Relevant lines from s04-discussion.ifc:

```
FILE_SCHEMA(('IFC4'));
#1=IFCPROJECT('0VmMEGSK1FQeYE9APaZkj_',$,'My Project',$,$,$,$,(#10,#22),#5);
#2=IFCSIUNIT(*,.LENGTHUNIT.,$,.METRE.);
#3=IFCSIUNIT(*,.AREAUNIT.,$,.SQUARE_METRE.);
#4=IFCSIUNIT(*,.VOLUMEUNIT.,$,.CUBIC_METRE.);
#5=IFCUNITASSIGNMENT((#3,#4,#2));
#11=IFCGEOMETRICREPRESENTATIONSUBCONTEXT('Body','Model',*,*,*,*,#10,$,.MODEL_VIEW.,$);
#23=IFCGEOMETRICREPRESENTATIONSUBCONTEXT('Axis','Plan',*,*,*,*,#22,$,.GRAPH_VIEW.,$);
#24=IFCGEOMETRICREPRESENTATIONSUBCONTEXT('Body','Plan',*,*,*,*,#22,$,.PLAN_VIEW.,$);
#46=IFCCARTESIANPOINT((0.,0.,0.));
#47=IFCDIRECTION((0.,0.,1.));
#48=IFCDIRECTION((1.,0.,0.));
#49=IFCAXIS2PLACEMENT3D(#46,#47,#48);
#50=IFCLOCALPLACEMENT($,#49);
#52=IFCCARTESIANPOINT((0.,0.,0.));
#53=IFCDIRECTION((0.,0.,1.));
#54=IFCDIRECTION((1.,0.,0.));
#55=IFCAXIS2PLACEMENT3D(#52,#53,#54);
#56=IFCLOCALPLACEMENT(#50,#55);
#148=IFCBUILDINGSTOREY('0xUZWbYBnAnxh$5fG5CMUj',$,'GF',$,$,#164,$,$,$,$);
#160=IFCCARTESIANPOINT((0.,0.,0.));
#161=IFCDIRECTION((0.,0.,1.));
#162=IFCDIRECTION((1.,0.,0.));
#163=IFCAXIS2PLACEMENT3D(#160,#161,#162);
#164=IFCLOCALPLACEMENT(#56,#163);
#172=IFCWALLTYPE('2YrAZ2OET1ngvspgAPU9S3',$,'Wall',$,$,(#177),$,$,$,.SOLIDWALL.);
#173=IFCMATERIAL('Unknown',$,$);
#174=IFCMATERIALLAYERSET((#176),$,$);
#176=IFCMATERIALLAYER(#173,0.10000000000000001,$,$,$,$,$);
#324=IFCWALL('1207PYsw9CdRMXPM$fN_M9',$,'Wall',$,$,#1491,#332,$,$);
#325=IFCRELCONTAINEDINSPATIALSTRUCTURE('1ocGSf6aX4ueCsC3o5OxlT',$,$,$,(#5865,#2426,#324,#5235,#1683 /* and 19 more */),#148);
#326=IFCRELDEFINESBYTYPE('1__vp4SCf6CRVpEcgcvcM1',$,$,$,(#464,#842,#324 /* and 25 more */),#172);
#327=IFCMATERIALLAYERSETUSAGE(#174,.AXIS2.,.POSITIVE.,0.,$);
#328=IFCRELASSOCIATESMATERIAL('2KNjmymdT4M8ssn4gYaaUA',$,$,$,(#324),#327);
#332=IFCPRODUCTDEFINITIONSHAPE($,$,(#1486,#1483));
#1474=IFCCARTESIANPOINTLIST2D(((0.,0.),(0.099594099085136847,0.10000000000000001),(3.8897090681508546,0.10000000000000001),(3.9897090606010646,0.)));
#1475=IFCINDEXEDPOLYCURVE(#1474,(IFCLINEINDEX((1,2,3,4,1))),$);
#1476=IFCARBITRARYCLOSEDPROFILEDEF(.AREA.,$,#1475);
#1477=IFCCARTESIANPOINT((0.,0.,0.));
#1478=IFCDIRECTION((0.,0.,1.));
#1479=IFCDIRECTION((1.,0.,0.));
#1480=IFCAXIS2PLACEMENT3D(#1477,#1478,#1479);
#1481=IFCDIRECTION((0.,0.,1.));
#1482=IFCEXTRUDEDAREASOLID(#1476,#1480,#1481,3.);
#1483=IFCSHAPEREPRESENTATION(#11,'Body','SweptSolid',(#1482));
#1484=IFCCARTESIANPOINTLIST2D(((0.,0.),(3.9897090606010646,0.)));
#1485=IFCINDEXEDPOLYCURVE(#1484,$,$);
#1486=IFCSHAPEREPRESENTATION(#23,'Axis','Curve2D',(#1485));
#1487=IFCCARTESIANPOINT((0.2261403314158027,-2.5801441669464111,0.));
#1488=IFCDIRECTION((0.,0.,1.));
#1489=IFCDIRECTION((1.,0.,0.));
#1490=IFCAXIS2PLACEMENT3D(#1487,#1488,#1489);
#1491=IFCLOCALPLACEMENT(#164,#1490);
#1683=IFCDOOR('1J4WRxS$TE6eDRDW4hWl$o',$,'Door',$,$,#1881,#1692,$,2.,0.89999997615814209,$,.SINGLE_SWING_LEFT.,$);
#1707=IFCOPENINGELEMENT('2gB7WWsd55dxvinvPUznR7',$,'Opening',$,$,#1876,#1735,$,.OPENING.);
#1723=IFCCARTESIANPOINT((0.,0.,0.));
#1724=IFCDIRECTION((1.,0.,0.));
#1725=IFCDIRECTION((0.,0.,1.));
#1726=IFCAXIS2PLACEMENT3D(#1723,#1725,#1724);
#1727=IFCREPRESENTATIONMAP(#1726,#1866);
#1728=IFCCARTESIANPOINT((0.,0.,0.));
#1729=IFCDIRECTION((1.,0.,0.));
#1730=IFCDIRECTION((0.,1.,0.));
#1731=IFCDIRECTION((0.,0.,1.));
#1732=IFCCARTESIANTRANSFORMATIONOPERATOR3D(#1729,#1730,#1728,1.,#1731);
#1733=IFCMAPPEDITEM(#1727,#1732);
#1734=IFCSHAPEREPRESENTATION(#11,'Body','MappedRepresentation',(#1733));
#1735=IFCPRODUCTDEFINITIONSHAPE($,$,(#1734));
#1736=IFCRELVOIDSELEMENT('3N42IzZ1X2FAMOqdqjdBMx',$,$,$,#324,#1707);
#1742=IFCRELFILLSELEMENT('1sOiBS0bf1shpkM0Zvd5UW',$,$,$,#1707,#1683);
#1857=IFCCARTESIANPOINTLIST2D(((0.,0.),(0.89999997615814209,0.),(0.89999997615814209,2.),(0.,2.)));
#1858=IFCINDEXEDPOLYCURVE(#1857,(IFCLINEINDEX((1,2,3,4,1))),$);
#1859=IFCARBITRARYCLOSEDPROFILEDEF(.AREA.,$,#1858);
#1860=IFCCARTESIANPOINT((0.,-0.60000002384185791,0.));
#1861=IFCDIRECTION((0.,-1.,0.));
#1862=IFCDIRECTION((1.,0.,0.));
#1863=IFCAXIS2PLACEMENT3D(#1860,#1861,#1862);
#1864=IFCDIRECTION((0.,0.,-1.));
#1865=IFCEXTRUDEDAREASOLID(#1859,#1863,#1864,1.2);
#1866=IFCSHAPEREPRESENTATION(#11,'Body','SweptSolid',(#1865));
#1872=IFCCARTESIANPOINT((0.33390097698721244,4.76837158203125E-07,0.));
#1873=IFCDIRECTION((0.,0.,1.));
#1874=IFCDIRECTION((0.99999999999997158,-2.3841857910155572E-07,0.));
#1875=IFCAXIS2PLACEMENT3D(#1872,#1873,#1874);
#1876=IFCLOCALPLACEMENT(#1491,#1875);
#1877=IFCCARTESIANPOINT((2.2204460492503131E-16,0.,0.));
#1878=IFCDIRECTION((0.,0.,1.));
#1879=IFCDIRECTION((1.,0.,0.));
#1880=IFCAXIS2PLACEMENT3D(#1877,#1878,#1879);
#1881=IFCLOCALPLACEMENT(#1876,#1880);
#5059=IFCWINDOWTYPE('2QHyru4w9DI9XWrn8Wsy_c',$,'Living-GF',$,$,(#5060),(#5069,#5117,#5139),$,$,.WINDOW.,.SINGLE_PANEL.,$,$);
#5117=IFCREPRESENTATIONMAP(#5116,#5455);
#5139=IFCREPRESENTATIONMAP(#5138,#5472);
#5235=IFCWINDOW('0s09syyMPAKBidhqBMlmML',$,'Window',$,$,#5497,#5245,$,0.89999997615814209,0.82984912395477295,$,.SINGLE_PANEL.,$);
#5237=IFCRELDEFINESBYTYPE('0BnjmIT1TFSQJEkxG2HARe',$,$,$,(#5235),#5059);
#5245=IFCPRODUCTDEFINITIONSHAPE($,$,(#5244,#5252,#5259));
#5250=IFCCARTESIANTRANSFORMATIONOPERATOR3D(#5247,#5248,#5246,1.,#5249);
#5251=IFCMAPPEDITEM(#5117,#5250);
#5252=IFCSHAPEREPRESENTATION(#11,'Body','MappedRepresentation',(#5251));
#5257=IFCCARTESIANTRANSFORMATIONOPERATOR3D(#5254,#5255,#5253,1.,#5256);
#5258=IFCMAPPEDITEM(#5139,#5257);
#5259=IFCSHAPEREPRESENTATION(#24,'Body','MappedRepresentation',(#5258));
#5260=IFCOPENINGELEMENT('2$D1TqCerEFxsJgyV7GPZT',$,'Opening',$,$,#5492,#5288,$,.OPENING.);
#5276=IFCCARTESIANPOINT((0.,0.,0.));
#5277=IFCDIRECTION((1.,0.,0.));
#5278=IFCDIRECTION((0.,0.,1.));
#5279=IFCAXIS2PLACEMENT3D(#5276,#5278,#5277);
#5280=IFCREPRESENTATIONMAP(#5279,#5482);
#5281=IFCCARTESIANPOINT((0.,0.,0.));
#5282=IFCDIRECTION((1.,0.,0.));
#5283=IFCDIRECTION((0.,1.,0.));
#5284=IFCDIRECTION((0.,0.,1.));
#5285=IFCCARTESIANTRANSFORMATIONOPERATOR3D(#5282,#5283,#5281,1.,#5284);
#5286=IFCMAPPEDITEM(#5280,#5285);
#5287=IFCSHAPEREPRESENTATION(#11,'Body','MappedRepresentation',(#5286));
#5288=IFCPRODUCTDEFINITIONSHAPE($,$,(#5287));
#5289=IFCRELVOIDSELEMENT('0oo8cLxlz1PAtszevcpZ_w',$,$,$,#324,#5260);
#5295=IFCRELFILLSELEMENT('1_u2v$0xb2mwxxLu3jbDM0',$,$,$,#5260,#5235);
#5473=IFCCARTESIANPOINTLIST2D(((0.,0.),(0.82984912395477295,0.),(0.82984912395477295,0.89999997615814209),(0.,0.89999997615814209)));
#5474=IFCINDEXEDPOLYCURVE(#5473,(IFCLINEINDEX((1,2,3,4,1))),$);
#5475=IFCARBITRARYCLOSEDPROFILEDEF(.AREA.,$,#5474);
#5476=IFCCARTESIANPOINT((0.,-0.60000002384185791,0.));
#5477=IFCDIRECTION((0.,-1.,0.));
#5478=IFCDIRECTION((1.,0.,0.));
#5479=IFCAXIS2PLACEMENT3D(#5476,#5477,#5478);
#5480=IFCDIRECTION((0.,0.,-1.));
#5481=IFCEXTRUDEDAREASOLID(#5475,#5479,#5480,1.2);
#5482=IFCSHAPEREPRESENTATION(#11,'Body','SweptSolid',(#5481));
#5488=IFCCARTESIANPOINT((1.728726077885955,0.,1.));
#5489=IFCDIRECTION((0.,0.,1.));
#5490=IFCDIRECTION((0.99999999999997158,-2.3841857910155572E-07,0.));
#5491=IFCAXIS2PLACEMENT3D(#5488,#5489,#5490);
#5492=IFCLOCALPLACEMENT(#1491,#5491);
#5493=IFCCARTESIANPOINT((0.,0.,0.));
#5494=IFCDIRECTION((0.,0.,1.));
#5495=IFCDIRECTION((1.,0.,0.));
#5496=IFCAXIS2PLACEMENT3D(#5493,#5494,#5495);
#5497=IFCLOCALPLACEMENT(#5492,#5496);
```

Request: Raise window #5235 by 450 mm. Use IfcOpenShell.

```python
import numpy as np
import ifcopenshell
import ifcopenshell.api.geometry
import ifcopenshell.util.placement
import ifcopenshell.util.unit

model = ifcopenshell.open("s04-discussion.ifc")
unit_scale = ifcopenshell.util.unit.calculate_unit_scale(model)

window = model.by_guid("0s09syyMPAKBidhqBMlmML")
opening = window.FillsVoids[0].RelatingOpeningElement
dz = 0.45 / unit_scale

shift = np.array([0.0, 0.0, dz])
# The window is placed relative to its opening, so it follows when the opening moves.
matrix = ifcopenshell.util.placement.get_local_placement(opening.ObjectPlacement)
matrix[:3, 3] += shift
ifcopenshell.api.geometry.edit_object_placement(
    model, product=opening, matrix=matrix, is_si=False, should_transform_children=True
)

print(f"moved by {dz * unit_scale:+.3f} m")

model.write("s04-discussion_updated.ifc")
```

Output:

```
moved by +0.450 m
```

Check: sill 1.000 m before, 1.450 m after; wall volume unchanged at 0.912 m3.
